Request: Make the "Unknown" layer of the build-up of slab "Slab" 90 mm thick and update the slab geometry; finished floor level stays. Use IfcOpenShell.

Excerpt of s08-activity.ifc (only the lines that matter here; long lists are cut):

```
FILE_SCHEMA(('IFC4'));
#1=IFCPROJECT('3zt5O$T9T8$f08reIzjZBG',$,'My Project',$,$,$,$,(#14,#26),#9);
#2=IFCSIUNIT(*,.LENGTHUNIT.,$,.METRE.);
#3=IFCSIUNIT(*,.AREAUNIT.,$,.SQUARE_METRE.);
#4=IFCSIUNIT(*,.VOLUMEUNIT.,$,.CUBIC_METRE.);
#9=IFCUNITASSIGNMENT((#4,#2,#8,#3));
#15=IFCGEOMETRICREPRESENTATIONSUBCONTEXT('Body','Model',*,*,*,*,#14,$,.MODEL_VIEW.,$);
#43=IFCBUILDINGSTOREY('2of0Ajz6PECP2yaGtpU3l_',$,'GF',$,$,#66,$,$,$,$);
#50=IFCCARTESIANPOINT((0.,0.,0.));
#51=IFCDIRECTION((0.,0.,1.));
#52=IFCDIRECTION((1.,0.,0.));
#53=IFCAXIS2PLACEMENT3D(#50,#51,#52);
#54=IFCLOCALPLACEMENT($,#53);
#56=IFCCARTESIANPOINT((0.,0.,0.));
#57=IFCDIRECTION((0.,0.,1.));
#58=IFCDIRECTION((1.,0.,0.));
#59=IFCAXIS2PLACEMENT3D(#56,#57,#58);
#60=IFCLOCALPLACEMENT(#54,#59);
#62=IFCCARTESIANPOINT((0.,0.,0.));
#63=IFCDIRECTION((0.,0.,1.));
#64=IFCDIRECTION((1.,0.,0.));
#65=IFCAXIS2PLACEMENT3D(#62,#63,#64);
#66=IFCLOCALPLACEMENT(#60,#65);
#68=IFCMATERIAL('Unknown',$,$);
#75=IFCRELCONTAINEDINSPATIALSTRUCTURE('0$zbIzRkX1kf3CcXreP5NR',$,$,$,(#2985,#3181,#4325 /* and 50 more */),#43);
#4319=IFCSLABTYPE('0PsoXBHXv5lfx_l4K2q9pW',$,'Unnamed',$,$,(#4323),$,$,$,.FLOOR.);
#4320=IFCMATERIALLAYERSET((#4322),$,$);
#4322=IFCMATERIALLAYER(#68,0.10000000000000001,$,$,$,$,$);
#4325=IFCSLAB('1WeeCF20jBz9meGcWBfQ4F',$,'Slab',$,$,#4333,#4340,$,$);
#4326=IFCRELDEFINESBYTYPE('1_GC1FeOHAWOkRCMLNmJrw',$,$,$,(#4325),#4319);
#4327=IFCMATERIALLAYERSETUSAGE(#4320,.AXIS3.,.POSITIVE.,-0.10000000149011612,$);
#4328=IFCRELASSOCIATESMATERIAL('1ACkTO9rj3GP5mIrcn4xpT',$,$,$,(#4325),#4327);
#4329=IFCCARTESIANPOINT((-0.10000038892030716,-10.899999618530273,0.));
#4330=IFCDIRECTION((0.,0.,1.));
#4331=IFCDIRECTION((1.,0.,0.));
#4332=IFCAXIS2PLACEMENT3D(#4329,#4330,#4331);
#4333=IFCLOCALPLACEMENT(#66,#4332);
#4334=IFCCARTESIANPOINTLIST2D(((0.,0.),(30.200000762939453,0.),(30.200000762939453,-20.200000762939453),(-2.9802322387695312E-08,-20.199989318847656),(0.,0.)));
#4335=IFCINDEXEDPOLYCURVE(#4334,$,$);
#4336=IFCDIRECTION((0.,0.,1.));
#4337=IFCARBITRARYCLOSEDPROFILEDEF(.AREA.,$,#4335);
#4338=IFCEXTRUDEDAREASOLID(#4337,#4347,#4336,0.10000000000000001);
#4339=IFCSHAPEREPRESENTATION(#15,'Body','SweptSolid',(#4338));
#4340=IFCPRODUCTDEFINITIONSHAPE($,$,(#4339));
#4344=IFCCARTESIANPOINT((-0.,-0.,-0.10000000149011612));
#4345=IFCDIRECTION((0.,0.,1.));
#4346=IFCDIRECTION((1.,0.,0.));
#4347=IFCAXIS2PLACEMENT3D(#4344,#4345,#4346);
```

```python
import ifcopenshell
import ifcopenshell.util.element
import ifcopenshell.util.representation
import ifcopenshell.util.unit

model = ifcopenshell.open("s08-activity.ifc")
unit_scale = ifcopenshell.util.unit.calculate_unit_scale(model)

layer_set = model.by_id(4320)
layer = next(l for l in layer_set.MaterialLayers if l.Material and l.Material.Name == "Unknown")
change = 0.09 / unit_scale - layer.LayerThickness
layer.LayerThickness += change

# Geometry does not follow the layer set by itself.
slabs = [e for e in ifcopenshell.util.element.get_elements_by_material(model, layer_set) if e.is_a("IfcSlab")]
for slab in sorted(slabs, key=lambda e: e.id()):
    body = ifcopenshell.util.representation.get_representation(slab, "Model", "Body")
    solid = body.Items[0]
    old_depth = solid.Depth
    solid.Depth += change
    # Extruded upwards: lower the start of the extrusion so the top stays.
    x, y, z = solid.Position.Location.Coordinates
    solid.Position.Location = model.createIfcCartesianPoint((x, y, z - change))
    print(slab.id(), f"{old_depth:g} -> {solid.Depth:g}")

# The layers are counted up from the underside, which has moved.
for usage in {ifcopenshell.util.element.get_material(slab) for slab in slabs}:
    usage.OffsetFromReferenceLine -= change

model.write("s08-activity_rev.ifc")
```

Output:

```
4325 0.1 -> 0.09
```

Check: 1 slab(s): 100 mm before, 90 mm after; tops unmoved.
